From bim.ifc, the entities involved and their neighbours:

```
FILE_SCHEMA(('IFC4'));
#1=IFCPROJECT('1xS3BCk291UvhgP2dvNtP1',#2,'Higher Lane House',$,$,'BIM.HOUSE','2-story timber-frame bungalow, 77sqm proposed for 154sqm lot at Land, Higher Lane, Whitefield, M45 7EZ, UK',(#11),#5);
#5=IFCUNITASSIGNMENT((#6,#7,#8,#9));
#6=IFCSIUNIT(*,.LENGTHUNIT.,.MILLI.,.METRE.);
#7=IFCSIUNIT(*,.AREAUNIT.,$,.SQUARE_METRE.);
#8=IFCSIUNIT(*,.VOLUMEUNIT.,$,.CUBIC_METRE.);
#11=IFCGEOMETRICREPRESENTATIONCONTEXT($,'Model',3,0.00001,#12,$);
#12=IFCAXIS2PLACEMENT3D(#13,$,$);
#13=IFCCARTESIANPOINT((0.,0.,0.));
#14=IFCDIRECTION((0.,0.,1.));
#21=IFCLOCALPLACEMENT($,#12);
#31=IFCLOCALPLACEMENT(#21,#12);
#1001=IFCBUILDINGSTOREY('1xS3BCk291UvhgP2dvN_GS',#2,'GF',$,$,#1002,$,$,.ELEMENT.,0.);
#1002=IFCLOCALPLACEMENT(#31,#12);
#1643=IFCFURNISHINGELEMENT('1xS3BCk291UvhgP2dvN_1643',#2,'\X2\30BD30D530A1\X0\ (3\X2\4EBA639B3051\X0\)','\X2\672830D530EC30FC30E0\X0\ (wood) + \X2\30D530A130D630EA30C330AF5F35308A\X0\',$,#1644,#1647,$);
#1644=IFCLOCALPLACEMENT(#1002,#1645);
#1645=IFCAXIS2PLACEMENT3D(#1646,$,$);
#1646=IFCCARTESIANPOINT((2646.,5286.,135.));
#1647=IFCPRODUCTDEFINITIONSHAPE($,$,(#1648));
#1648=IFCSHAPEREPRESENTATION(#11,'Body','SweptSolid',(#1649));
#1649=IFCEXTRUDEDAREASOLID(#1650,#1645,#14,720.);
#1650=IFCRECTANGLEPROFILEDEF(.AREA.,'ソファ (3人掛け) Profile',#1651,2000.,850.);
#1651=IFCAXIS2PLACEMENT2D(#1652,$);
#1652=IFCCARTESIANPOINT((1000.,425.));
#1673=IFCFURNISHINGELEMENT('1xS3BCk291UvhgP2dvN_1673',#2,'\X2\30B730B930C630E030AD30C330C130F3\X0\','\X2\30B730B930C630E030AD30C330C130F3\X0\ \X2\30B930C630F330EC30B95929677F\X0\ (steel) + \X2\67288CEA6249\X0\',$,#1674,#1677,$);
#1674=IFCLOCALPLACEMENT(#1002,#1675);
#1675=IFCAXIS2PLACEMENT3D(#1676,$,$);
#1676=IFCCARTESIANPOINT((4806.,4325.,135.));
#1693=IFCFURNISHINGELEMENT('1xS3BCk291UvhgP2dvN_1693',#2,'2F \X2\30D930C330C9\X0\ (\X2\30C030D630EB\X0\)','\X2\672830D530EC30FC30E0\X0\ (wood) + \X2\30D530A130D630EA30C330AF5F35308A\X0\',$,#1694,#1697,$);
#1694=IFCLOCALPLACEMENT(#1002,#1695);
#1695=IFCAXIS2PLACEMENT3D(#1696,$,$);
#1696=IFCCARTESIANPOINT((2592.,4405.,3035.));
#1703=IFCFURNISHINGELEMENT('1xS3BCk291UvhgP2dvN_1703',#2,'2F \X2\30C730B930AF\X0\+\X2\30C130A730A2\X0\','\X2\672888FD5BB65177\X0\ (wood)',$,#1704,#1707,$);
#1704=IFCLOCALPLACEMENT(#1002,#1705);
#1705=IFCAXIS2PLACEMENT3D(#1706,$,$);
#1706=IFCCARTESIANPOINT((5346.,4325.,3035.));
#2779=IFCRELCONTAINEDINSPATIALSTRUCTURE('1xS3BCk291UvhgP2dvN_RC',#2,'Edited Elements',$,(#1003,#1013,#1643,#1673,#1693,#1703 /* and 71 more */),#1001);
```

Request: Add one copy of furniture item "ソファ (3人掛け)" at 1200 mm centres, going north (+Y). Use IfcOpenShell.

```python
import numpy as np
import ifcopenshell
import ifcopenshell.api.geometry
import ifcopenshell.api.root
import ifcopenshell.util.element
import ifcopenshell.util.placement

model = ifcopenshell.open("bim.ifc")


def reuse_history(source, copy):
    """copy_class also copies each property set's owner history, people and application; keep the originals."""
    for rel in copy.IsDefinedBy:
        if rel.is_a("IfcRelDefinesByProperties") and (history := rel.RelatingPropertyDefinition.OwnerHistory):
            rel.RelatingPropertyDefinition.OwnerHistory = source.OwnerHistory
            ifcopenshell.util.element.remove_deep2(model, history)


source = model.by_guid("1xS3BCk291UvhgP2dvN_1643")
base = ifcopenshell.util.placement.get_local_placement(source.ObjectPlacement)
step = np.array([0.0, 1.0, 0.0]) * 1200.0

for i in range(1, 2):
    copy = ifcopenshell.api.root.copy_class(model, product=source)
    copy.Representation = ifcopenshell.util.element.copy_deep(
        model, source.Representation, exclude=["IfcGeometricRepresentationContext", "IfcRepresentationMap"]
    )
    reuse_history(source, copy)
    matrix = base.copy()
    matrix[:3, 3] += i * step
    print("added at", matrix[:3, 3].round(3) + 0.0)
    ifcopenshell.api.geometry.edit_object_placement(model, product=copy, matrix=matrix, is_si=False)

model.write("bim_rev.ifc")
```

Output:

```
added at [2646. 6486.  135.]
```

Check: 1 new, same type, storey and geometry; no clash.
